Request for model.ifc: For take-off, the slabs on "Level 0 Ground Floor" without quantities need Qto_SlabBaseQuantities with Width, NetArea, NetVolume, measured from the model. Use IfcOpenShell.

First a look at what the model holds.

```python
import ifcopenshell
import ifcopenshell.util.element
import ifcopenshell.util.unit

model = ifcopenshell.open("model.ifc")
print(model.schema)
for unit_type in ("LENGTHUNIT", "AREAUNIT", "VOLUMEUNIT"):
    print(unit_type, ifcopenshell.util.unit.calculate_unit_scale(model, unit_type))
storey = next(s for s in model.by_type("IfcBuildingStorey") if s.Name == "Level 0 Ground Floor")
slabs = [e for e in ifcopenshell.util.element.get_decomposition(storey) if e.is_a("IfcSlab")]
for e in sorted(slabs, key=lambda e: e.id()):
    print(e.id(), e.is_a(), e.Name, list(ifcopenshell.util.element.get_psets(e, qtos_only=True)), sep=" | ")
```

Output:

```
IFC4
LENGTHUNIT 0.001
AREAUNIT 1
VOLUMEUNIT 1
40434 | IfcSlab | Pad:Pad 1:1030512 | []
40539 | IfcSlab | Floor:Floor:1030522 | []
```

```python
import ifcopenshell
import ifcopenshell.api.pset
import ifcopenshell.geom
import ifcopenshell.util.element
import ifcopenshell.util.shape
import ifcopenshell.util.unit

model = ifcopenshell.open("model.ifc")
unit_scale = ifcopenshell.util.unit.calculate_unit_scale(model)
area_scale = ifcopenshell.util.unit.calculate_unit_scale(model, "AREAUNIT")
volume_scale = ifcopenshell.util.unit.calculate_unit_scale(model, "VOLUMEUNIT")
settings = ifcopenshell.geom.settings()

storey = next(s for s in model.by_type("IfcBuildingStorey") if s.Name == "Level 0 Ground Floor")
slabs = [e for e in ifcopenshell.util.element.get_decomposition(storey) if e.is_a("IfcSlab")]

for e in sorted(slabs, key=lambda e: e.id()):
    if ifcopenshell.util.element.get_psets(e, qtos_only=True, should_inherit=False):
        continue
    # Geometry comes back in metres, in the element's own axes.
    shape = ifcopenshell.geom.create_shape(settings, e)
    values = {
        "Width": ifcopenshell.util.shape.get_z(shape.geometry) / unit_scale,
        "NetArea": ifcopenshell.util.shape.get_footprint_area(shape.geometry) / area_scale,
        "NetVolume": ifcopenshell.util.shape.get_volume(shape.geometry) / volume_scale,
    }
    qto = ifcopenshell.api.pset.add_qto(model, product=e, name="Qto_SlabBaseQuantities")
    ifcopenshell.api.pset.edit_qto(model, qto=qto, properties=values)
    print(e.id(), {k: round(v, 3) for k, v in values.items()})

model.write("model_edited.ifc")
```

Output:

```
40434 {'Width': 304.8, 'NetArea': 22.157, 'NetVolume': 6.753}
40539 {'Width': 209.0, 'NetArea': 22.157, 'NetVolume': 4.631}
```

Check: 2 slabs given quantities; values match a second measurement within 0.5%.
